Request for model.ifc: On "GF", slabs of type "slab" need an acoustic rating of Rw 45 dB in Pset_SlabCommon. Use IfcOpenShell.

First a look at what the model holds.

```python
import ifcopenshell
import ifcopenshell.util.element

model = ifcopenshell.open("model.ifc")
print(model.schema)
storey = next(s for s in model.by_type("IfcBuildingStorey") if s.Name == "GF")
slabs = [e for e in ifcopenshell.util.element.get_decomposition(storey) if e.is_a("IfcSlab")]
seen = {}
for e in slabs:
    element_type = ifcopenshell.util.element.get_type(e)
    key = (element_type.Name if element_type != e and element_type else None, ifcopenshell.util.element.get_pset(e, "Pset_SlabCommon", "AcousticRating"))
    seen[key] = seen.get(key, 0) + 1
for (name, value), count in sorted(seen.items(), key=str):
    print(count, "x", name, "|", value)
```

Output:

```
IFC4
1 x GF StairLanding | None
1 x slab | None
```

```python
import ifcopenshell
import ifcopenshell.api.pset
import ifcopenshell.util.element

model = ifcopenshell.open("model.ifc")

storey = next(s for s in model.by_type("IfcBuildingStorey") if s.Name == "GF")
slabs = [e for e in ifcopenshell.util.element.get_decomposition(storey) if e.is_a("IfcSlab")]

count = 0
for e in slabs:
    element_type = ifcopenshell.util.element.get_type(e)
    if element_type in (None, e) or element_type.Name != "slab":
        continue
    # add_pset returns the element's existing set when there is one.
    pset = ifcopenshell.api.pset.add_pset(model, product=e, name="Pset_SlabCommon")
    ifcopenshell.api.pset.edit_pset(model, pset=pset, properties={"AcousticRating": "Rw 45 dB"})
    count += 1

print(count, "slabs updated")

model.write("model_edited.ifc")
```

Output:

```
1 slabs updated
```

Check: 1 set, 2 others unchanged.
